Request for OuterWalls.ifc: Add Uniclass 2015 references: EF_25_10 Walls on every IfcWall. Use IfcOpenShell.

First a look at what the model holds.

```python
import ifcopenshell

model = ifcopenshell.open("OuterWalls.ifc")
print(model.schema)
print("classifications:", [c.Name for c in model.by_type("IfcClassification")])
for ifc_class in ("IfcDoor", "IfcRoof", "IfcStair", "IfcWall", "IfcWindow"):
    print(ifc_class, len(model.by_type(ifc_class)))
```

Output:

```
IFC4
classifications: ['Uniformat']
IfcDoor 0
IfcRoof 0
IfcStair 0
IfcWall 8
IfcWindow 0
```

```python
import ifcopenshell
import ifcopenshell.api.classification

model = ifcopenshell.open("OuterWalls.ifc")

system = ifcopenshell.api.classification.add_classification(model, classification="Uniclass 2015")

codes = {
    "IfcWall": ("EF_25_10", "Walls"),
}
for ifc_class, (code, name) in codes.items():
    products = model.by_type(ifc_class)
    ifcopenshell.api.classification.add_reference(
        model, products=products, classification=system, identification=code, name=name
    )
    print(code, len(products))

model.write("OuterWalls_v2.ifc")
```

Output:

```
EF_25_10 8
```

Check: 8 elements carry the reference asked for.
